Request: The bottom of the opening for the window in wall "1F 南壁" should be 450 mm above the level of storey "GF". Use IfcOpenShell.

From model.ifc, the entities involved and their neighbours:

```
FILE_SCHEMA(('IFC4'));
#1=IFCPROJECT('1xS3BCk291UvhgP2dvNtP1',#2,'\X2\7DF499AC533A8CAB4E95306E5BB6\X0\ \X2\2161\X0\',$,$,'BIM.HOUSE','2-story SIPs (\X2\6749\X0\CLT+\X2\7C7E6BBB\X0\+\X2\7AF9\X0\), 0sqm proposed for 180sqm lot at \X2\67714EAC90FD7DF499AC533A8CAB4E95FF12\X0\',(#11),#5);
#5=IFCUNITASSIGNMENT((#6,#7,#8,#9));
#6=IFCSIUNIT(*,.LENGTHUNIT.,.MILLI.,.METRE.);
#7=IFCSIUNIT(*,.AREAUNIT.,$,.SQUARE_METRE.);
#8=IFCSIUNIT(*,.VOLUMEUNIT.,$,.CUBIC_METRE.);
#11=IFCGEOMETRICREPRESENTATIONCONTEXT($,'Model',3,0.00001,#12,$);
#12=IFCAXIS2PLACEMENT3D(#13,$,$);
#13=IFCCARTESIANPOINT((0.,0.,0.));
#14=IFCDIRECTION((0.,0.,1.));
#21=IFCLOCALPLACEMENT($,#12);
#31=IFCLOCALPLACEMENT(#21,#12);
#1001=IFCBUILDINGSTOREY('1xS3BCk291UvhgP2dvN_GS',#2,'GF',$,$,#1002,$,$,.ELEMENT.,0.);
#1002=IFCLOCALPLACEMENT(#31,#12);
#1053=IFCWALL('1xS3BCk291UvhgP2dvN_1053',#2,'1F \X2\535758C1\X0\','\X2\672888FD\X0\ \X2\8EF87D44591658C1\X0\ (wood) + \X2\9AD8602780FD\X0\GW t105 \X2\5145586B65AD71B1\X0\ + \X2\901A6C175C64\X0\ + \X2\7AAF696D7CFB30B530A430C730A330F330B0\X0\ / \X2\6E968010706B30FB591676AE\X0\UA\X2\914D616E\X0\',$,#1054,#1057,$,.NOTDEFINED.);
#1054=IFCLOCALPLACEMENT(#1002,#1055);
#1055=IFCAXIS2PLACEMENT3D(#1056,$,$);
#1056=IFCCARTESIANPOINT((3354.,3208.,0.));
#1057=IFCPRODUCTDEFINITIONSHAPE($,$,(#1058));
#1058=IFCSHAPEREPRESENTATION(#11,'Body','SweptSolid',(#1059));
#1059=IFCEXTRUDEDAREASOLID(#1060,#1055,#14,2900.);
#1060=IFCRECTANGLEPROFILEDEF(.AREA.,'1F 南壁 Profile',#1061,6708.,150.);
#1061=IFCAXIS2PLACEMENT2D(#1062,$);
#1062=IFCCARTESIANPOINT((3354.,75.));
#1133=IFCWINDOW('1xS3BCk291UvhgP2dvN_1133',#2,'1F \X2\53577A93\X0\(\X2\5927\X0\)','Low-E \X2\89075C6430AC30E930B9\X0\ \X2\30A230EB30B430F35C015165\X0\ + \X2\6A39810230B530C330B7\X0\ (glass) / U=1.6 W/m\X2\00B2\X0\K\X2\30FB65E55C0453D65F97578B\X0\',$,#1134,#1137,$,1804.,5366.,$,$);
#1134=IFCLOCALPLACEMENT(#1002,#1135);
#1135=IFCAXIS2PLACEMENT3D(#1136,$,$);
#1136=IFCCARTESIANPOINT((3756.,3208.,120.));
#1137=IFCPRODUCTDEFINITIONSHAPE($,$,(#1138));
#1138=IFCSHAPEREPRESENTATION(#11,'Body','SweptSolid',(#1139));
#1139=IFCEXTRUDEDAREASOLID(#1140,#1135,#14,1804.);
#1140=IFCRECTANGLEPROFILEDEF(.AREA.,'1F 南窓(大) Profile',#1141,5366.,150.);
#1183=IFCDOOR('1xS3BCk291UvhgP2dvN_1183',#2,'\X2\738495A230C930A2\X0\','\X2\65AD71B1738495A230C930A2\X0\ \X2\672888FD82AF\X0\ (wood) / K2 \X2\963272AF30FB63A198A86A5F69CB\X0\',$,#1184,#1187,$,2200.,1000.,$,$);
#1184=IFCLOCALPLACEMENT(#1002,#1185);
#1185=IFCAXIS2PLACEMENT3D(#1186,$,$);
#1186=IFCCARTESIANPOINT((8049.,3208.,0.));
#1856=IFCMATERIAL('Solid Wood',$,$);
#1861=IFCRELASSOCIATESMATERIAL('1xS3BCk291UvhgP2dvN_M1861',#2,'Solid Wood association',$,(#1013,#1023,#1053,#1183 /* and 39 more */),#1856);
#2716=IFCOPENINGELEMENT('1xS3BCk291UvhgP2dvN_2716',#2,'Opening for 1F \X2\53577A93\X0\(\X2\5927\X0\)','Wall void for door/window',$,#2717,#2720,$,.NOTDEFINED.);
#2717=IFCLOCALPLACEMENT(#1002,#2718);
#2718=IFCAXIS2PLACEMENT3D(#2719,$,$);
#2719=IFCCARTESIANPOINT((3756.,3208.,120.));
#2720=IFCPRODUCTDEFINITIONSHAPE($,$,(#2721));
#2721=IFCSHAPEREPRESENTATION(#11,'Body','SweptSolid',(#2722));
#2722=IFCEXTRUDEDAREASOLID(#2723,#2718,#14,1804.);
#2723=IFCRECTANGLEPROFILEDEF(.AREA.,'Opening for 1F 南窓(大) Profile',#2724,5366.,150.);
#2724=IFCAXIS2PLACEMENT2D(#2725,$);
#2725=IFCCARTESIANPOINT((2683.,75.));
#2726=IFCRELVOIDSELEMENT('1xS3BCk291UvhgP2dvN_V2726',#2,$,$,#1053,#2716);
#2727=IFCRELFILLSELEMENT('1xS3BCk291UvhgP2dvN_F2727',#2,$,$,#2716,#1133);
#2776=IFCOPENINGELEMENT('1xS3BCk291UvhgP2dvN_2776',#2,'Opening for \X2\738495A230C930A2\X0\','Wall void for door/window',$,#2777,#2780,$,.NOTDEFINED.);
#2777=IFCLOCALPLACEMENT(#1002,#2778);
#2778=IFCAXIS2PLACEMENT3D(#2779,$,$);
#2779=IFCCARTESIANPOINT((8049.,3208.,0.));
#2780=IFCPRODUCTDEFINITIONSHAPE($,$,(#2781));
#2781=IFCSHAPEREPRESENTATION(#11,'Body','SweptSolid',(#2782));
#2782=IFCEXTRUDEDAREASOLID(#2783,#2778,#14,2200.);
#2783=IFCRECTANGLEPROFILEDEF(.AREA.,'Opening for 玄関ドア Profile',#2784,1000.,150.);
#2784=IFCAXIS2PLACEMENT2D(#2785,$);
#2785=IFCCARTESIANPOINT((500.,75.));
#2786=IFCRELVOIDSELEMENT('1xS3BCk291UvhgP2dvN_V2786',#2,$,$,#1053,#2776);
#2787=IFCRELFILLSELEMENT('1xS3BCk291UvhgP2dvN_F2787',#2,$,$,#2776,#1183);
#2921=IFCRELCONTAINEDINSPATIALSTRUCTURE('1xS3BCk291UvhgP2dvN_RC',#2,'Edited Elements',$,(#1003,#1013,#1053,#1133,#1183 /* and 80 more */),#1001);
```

```python
import numpy as np
import ifcopenshell
import ifcopenshell.api.geometry
import ifcopenshell.geom
import ifcopenshell.util.element
import ifcopenshell.util.placement
import ifcopenshell.util.shape
import ifcopenshell.util.unit

model = ifcopenshell.open("model.ifc")
unit_scale = ifcopenshell.util.unit.calculate_unit_scale(model)

window = model.by_guid("1xS3BCk291UvhgP2dvN_1133")
opening = window.FillsVoids[0].RelatingOpeningElement
storey = ifcopenshell.util.element.get_container(window, ifc_class="IfcBuildingStorey")
level = ifcopenshell.util.placement.get_local_placement(storey.ObjectPlacement)[2, 3]

# The opening's origin need not be at the sill, so measure its lowest point.
shape = ifcopenshell.geom.create_shape(ifcopenshell.geom.settings(), opening)
bottom = ifcopenshell.util.shape.get_shape_bottom_elevation(shape, shape.geometry) / unit_scale
dz = level + 0.45 / unit_scale - bottom

shift = np.array([0.0, 0.0, dz])
# The window is not placed relative to its opening, so move both.
for product in (opening, window):
    matrix = ifcopenshell.util.placement.get_local_placement(product.ObjectPlacement)
    matrix[:3, 3] += shift
    ifcopenshell.api.geometry.edit_object_placement(model, product=product, matrix=matrix, is_si=False)

print(f"moved by {dz * unit_scale:+.3f} m")

model.write("model-out.ifc")
```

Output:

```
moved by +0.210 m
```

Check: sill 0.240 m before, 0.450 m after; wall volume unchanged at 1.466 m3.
